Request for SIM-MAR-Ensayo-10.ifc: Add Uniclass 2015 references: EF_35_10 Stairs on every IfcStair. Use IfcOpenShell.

First a look at what the model holds.

```python
import ifcopenshell

model = ifcopenshell.open("SIM-MAR-Ensayo-10.ifc")
print(model.schema)
print("classifications:", [c.Name for c in model.by_type("IfcClassification")])
for ifc_class in ("IfcDoor", "IfcRoof", "IfcStair", "IfcWall", "IfcWindow"):
    print(ifc_class, len(model.by_type(ifc_class)))
```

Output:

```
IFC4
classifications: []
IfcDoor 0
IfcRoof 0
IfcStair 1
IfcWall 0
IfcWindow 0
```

```python
import ifcopenshell
import ifcopenshell.api.classification

model = ifcopenshell.open("SIM-MAR-Ensayo-10.ifc")

system = ifcopenshell.api.classification.add_classification(model, classification="Uniclass 2015")

codes = {
    "IfcStair": ("EF_35_10", "Stairs"),
}
for ifc_class, (code, name) in codes.items():
    products = model.by_type(ifc_class)
    ifcopenshell.api.classification.add_reference(
        model, products=products, classification=system, identification=code, name=name
    )
    print(code, len(products))

model.write("SIM-MAR-Ensayo-10-out.ifc")
```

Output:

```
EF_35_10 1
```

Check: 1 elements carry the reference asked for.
